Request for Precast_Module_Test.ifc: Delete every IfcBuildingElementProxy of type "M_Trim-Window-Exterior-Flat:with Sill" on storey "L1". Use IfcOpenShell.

First a look at what the model holds.

```python
import ifcopenshell
import ifcopenshell.util.element

model = ifcopenshell.open("Precast_Module_Test.ifc")
print(model.schema)
storey = next(s for s in model.by_type("IfcBuildingStorey") if s.Name == "L1")
proxies = [e for e in ifcopenshell.util.element.get_decomposition(storey) if e.is_a("IfcBuildingElementProxy")]
seen = {}
for e in proxies:
    element_type = ifcopenshell.util.element.get_type(e)
    name = element_type.Name if element_type not in (None, e) else None
    seen[name] = seen.get(name, 0) + 1
for name, count in sorted(seen.items(), key=str):
    print(count, "x", name)
```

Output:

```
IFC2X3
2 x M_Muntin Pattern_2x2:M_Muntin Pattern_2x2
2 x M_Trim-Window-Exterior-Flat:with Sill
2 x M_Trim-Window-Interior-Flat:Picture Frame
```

```python
import ifcopenshell
import ifcopenshell.api.root
import ifcopenshell.util.element

model = ifcopenshell.open("Precast_Module_Test.ifc")

storey = next(s for s in model.by_type("IfcBuildingStorey") if s.Name == "L1")
proxies = [e for e in ifcopenshell.util.element.get_decomposition(storey) if e.is_a("IfcBuildingElementProxy")]
targets = [e for e in proxies if (t := ifcopenshell.util.element.get_type(e)) not in (None, e) and t.Name == "M_Trim-Window-Exterior-Flat:with Sill"]

for e in targets:
    ifcopenshell.api.root.remove_product(model, product=e)
print(len(targets), "removed")

model.write("Precast_Module_Test_rev.ifc")
```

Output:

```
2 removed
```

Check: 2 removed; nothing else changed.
